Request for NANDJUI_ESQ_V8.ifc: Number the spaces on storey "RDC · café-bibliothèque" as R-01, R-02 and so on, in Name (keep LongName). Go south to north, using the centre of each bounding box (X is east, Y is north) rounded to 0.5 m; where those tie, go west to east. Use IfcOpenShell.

First a look at what the model holds.

```python
import ifcopenshell
import ifcopenshell.util.element
import ifcopenshell.util.placement

model = ifcopenshell.open("NANDJUI_ESQ_V8.ifc")
print(model.schema)
storey = next(s for s in model.by_type("IfcBuildingStorey") if s.Name == "RDC · café-bibliothèque")
spaces = [e for e in ifcopenshell.util.element.get_decomposition(storey) if e.is_a("IfcSpace")]
for e in sorted(spaces, key=lambda e: e.id()):
    origin = ifcopenshell.util.placement.get_local_placement(e.ObjectPlacement)[:3, 3]
    print(e.id(), e.Name, e.LongName, origin.round(2) + 0.0, sep=" | ")
```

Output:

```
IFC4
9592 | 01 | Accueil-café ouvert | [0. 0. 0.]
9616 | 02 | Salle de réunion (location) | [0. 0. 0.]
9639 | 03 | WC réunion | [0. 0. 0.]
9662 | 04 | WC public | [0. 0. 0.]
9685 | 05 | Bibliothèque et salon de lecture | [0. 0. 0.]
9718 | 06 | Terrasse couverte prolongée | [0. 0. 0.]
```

```python
import ifcopenshell
import ifcopenshell.geom
import ifcopenshell.util.element
import ifcopenshell.util.shape

model = ifcopenshell.open("NANDJUI_ESQ_V8.ifc")
settings = ifcopenshell.geom.settings()
settings.set("use-world-coords", True)


def centre(element):
    shape = ifcopenshell.geom.create_shape(settings, element)
    return ifcopenshell.util.shape.get_bbox_centroid(shape.geometry)


storey = next(s for s in model.by_type("IfcBuildingStorey") if s.Name == "RDC · café-bibliothèque")
spaces = [e for e in ifcopenshell.util.element.get_decomposition(storey) if e.is_a("IfcSpace")]

# Insertion points can sit at a corner or the storey origin, so sort by the geometry (in metres).
centres = {e: centre(e) for e in spaces}
spaces.sort(key=lambda e: (round(centres[e][1] / 0.5), centres[e][0]))

for i, e in enumerate(spaces, start=1):
    number = f"R-{i:02d}"
    e.Name = number
    print(e.id(), number)

model.write("NANDJUI_ESQ_V8_rev.ifc")
```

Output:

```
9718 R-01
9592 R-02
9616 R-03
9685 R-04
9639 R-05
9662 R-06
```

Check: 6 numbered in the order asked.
